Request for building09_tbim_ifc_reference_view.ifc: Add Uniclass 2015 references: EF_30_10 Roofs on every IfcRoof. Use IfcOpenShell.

First a look at what the model holds.

```python
import ifcopenshell

model = ifcopenshell.open("building09_tbim_ifc_reference_view.ifc")
print(model.schema)
print("classifications:", [c.Name for c in model.by_type("IfcClassification")])
for ifc_class in ("IfcDoor", "IfcRoof", "IfcStair", "IfcWall", "IfcWindow"):
    print(ifc_class, len(model.by_type(ifc_class)))
```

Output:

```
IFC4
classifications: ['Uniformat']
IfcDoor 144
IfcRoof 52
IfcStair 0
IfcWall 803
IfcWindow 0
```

```python
import ifcopenshell
import ifcopenshell.api.classification

model = ifcopenshell.open("building09_tbim_ifc_reference_view.ifc")

system = ifcopenshell.api.classification.add_classification(model, classification="Uniclass 2015")

codes = {
    "IfcRoof": ("EF_30_10", "Roofs"),
}
for ifc_class, (code, name) in codes.items():
    products = model.by_type(ifc_class)
    ifcopenshell.api.classification.add_reference(
        model, products=products, classification=system, identification=code, name=name
    )
    print(code, len(products))

model.write("building09_tbim_ifc_reference_view_rev.ifc")
```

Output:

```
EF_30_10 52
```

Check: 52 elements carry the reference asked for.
